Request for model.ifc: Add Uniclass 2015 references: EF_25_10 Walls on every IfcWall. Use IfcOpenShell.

First a look at what the model holds.

```python
import ifcopenshell

model = ifcopenshell.open("model.ifc")
print(model.schema)
print("classifications:", [c.Name for c in model.by_type("IfcClassification")])
for ifc_class in ("IfcDoor", "IfcRoof", "IfcStair", "IfcWall", "IfcWindow"):
    print(ifc_class, len(model.by_type(ifc_class)))
```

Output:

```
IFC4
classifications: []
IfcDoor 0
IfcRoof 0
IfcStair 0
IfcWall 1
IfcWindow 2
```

```python
import ifcopenshell
import ifcopenshell.api.classification

model = ifcopenshell.open("model.ifc")

system = ifcopenshell.api.classification.add_classification(model, classification="Uniclass 2015")

codes = {
    "IfcWall": ("EF_25_10", "Walls"),
}
for ifc_class, (code, name) in codes.items():
    products = model.by_type(ifc_class)
    ifcopenshell.api.classification.add_reference(
        model, products=products, classification=system, identification=code, name=name
    )
    print(code, len(products))

model.write("model_rev.ifc")
```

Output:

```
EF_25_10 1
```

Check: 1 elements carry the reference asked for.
